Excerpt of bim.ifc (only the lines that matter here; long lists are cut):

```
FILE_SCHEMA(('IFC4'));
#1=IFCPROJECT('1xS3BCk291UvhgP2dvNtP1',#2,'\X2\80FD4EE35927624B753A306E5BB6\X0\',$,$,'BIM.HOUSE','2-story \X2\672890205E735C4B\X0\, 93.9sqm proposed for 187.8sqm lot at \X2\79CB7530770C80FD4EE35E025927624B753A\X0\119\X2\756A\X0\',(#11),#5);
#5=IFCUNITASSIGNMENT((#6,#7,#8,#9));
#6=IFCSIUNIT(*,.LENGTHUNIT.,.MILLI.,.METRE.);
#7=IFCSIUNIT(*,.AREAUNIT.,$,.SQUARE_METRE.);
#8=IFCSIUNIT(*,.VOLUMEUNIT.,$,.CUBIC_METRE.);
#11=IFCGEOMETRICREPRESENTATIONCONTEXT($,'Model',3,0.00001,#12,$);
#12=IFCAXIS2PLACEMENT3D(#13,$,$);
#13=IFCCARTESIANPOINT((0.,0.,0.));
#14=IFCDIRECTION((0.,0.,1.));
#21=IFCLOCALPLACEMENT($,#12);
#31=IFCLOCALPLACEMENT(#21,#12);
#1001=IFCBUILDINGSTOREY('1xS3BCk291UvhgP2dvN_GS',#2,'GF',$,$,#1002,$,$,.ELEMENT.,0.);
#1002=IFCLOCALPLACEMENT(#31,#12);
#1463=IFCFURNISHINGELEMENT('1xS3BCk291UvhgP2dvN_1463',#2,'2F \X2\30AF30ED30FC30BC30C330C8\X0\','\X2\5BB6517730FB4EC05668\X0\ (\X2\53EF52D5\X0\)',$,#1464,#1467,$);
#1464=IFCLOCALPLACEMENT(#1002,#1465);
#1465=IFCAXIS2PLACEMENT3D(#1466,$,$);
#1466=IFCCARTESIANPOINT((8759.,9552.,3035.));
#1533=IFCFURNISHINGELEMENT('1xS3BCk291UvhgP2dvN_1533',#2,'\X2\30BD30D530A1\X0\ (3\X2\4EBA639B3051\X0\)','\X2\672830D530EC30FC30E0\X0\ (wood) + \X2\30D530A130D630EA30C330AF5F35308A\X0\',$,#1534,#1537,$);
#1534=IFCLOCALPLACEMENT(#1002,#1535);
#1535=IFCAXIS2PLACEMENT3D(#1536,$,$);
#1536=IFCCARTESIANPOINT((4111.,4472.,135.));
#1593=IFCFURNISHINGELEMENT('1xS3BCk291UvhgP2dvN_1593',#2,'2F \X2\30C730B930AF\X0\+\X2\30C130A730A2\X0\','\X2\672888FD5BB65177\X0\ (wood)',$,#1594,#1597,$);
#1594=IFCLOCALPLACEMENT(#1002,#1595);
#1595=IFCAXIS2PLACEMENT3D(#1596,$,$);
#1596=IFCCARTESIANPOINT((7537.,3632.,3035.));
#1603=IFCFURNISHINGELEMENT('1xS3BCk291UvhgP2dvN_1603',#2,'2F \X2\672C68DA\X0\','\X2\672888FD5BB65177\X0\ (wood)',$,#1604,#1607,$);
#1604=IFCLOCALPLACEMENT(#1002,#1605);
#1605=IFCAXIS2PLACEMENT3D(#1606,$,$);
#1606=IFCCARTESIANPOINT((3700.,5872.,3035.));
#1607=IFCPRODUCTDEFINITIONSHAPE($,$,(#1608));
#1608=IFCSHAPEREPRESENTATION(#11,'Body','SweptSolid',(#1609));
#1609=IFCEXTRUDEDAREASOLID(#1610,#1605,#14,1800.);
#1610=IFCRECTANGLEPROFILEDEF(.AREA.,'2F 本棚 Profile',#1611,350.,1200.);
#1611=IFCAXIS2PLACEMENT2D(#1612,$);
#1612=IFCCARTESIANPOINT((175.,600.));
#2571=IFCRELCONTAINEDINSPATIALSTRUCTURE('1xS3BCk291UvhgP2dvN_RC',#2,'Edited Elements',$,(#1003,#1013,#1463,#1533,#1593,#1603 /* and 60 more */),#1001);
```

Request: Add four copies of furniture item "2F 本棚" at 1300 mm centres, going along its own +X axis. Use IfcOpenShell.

```python
import ifcopenshell
import ifcopenshell.api.geometry
import ifcopenshell.api.root
import ifcopenshell.util.element
import ifcopenshell.util.placement
import ifcopenshell.util.unit

model = ifcopenshell.open("bim.ifc")
unit_scale = ifcopenshell.util.unit.calculate_unit_scale(model)


def reuse_history(source, copy):
    """copy_class also copies each property set's owner history, people and application; keep the originals."""
    for rel in copy.IsDefinedBy:
        if rel.is_a("IfcRelDefinesByProperties") and (history := rel.RelatingPropertyDefinition.OwnerHistory):
            rel.RelatingPropertyDefinition.OwnerHistory = source.OwnerHistory
            ifcopenshell.util.element.remove_deep2(model, history)


source = model.by_guid("1xS3BCk291UvhgP2dvN_1603")
base = ifcopenshell.util.placement.get_local_placement(source.ObjectPlacement)
step = base[:3, 0] * 1.3 / unit_scale

for i in range(1, 5):
    copy = ifcopenshell.api.root.copy_class(model, product=source)
    copy.Representation = ifcopenshell.util.element.copy_deep(
        model, source.Representation, exclude=["IfcGeometricRepresentationContext", "IfcRepresentationMap"]
    )
    reuse_history(source, copy)
    matrix = base.copy()
    matrix[:3, 3] += i * step
    print("added at", matrix[:3, 3].round(3) + 0.0)
    ifcopenshell.api.geometry.edit_object_placement(model, product=copy, matrix=matrix, is_si=False)

model.write("bim_updated.ifc")
```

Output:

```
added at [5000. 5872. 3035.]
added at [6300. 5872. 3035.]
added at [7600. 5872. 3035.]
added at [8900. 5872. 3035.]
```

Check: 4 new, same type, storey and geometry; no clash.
